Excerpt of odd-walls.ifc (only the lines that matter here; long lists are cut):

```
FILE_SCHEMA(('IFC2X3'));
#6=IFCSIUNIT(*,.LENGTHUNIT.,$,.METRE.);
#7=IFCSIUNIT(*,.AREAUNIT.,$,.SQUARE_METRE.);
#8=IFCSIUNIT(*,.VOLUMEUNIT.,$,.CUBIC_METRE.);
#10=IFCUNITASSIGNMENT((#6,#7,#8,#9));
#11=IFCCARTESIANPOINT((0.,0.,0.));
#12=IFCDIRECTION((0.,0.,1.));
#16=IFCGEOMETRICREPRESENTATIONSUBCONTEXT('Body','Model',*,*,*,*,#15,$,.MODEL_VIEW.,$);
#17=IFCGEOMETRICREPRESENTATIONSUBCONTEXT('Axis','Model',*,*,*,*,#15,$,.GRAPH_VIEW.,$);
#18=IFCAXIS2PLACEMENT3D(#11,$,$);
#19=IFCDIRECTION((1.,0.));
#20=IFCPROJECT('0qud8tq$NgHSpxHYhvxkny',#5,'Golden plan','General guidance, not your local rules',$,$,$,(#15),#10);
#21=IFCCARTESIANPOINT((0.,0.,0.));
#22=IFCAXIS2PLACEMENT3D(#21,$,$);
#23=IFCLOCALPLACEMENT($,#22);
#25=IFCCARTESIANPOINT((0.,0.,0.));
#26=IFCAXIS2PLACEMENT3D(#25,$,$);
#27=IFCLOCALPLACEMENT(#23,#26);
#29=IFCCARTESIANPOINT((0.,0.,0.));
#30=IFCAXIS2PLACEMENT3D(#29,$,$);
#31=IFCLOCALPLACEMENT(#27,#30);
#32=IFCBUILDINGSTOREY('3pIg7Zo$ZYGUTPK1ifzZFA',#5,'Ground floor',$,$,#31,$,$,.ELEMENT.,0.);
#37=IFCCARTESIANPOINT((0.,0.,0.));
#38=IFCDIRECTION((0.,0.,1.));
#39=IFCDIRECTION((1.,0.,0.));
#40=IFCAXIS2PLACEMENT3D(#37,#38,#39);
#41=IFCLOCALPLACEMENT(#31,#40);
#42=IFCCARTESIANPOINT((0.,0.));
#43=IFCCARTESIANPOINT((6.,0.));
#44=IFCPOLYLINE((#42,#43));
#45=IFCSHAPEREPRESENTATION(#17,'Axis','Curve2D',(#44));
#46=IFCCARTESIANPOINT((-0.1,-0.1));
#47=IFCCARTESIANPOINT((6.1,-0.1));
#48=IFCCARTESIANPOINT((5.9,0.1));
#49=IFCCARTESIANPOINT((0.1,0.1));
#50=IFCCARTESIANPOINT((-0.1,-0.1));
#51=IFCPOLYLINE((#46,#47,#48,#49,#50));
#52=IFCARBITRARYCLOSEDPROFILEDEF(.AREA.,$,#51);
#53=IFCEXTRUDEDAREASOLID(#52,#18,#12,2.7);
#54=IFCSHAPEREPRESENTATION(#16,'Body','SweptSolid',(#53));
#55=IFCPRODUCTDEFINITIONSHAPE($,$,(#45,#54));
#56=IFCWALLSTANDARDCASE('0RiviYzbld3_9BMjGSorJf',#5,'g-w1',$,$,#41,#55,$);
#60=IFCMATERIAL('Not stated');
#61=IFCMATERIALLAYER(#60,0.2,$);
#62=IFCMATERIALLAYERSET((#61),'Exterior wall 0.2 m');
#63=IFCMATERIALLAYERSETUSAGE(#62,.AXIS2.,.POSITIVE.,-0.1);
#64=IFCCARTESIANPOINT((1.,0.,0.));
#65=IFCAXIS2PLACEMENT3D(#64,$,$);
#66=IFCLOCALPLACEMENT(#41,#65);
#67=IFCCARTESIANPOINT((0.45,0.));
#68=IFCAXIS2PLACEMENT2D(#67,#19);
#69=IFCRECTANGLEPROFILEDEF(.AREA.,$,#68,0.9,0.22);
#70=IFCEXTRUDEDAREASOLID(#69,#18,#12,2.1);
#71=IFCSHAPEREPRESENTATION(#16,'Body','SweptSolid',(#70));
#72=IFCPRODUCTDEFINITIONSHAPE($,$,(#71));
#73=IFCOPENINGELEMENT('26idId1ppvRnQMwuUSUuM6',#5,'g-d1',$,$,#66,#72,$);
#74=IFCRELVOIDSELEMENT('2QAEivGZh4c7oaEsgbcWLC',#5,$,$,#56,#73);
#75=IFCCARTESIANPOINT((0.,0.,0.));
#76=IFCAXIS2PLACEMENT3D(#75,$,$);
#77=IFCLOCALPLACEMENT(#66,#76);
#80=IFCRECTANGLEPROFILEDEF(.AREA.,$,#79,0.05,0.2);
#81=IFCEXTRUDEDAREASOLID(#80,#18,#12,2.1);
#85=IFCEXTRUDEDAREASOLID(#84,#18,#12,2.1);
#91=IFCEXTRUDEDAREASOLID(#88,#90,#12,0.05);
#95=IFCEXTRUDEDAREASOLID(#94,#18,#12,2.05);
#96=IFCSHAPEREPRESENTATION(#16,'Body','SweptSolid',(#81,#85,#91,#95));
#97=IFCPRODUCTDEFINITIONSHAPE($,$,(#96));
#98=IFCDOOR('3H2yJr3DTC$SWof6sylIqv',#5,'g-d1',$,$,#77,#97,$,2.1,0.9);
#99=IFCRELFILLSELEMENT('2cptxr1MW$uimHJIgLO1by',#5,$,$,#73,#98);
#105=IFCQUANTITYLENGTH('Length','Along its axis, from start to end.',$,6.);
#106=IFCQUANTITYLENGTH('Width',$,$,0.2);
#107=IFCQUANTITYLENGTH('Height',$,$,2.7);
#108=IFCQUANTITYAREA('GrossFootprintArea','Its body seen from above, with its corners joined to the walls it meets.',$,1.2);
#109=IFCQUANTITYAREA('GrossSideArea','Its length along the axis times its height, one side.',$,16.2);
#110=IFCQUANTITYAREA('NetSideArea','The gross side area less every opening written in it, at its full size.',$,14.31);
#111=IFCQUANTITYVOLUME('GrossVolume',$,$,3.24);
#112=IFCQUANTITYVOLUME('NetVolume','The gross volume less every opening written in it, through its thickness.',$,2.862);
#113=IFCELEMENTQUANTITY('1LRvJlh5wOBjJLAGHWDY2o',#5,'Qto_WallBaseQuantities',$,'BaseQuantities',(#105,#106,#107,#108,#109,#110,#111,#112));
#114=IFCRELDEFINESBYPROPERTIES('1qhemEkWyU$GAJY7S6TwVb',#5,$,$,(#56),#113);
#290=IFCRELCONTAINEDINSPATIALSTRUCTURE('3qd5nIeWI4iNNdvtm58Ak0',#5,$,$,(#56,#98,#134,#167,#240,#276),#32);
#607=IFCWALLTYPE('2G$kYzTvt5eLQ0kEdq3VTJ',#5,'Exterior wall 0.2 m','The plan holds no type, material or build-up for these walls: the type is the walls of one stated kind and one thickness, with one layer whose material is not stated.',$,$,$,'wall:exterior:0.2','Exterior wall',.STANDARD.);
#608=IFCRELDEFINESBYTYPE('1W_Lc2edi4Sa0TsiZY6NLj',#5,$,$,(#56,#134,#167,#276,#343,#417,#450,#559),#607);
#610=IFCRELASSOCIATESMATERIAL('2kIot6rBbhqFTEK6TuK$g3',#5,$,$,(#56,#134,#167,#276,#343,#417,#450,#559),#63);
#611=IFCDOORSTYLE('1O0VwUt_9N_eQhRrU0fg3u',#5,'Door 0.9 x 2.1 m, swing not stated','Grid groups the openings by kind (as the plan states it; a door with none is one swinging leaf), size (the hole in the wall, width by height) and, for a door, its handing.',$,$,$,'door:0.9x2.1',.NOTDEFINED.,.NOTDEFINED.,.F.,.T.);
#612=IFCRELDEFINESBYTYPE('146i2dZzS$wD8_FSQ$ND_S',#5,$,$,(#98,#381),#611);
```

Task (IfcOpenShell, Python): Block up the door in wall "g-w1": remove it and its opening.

```python
import ifcopenshell
import ifcopenshell.api.feature
import ifcopenshell.api.pset
import ifcopenshell.api.root
import ifcopenshell.geom
import ifcopenshell.util.element
import ifcopenshell.util.shape
import ifcopenshell.util.unit

model = ifcopenshell.open("odd-walls.ifc")
area_scale = ifcopenshell.util.unit.calculate_unit_scale(model, "AREAUNIT")
volume_scale = ifcopenshell.util.unit.calculate_unit_scale(model, "VOLUMEUNIT")
settings = ifcopenshell.geom.settings()


def volume(element):
    """Net volume in cubic metres, openings subtracted."""
    shape = ifcopenshell.geom.create_shape(settings, element)
    return ifcopenshell.util.shape.get_volume(shape.geometry)


door = model.by_id(98)
opening = door.FillsVoids[0].RelatingOpeningElement
wall = opening.VoidsElements[0].RelatingBuildingElement
before = volume(wall)

ifcopenshell.api.root.remove_product(model, product=door)
ifcopenshell.api.feature.remove_feature(model, feature=opening)

after = volume(wall)
thickness = 0.2  # wall thickness in metres

# Update the wall's stored quantities.
qto = model.by_id(ifcopenshell.util.element.get_pset(wall, "Qto_WallBaseQuantities", should_inherit=False)["id"])
ifcopenshell.api.pset.edit_qto(model, qto=qto, properties={
    "NetSideArea": after / thickness / area_scale,
    "NetVolume": after / volume_scale,
})

print(f"wall volume {before:.3f} -> {after:.3f} m3")

model.write("odd-walls-out.ifc")
```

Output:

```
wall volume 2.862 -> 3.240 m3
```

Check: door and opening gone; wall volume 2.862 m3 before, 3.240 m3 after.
